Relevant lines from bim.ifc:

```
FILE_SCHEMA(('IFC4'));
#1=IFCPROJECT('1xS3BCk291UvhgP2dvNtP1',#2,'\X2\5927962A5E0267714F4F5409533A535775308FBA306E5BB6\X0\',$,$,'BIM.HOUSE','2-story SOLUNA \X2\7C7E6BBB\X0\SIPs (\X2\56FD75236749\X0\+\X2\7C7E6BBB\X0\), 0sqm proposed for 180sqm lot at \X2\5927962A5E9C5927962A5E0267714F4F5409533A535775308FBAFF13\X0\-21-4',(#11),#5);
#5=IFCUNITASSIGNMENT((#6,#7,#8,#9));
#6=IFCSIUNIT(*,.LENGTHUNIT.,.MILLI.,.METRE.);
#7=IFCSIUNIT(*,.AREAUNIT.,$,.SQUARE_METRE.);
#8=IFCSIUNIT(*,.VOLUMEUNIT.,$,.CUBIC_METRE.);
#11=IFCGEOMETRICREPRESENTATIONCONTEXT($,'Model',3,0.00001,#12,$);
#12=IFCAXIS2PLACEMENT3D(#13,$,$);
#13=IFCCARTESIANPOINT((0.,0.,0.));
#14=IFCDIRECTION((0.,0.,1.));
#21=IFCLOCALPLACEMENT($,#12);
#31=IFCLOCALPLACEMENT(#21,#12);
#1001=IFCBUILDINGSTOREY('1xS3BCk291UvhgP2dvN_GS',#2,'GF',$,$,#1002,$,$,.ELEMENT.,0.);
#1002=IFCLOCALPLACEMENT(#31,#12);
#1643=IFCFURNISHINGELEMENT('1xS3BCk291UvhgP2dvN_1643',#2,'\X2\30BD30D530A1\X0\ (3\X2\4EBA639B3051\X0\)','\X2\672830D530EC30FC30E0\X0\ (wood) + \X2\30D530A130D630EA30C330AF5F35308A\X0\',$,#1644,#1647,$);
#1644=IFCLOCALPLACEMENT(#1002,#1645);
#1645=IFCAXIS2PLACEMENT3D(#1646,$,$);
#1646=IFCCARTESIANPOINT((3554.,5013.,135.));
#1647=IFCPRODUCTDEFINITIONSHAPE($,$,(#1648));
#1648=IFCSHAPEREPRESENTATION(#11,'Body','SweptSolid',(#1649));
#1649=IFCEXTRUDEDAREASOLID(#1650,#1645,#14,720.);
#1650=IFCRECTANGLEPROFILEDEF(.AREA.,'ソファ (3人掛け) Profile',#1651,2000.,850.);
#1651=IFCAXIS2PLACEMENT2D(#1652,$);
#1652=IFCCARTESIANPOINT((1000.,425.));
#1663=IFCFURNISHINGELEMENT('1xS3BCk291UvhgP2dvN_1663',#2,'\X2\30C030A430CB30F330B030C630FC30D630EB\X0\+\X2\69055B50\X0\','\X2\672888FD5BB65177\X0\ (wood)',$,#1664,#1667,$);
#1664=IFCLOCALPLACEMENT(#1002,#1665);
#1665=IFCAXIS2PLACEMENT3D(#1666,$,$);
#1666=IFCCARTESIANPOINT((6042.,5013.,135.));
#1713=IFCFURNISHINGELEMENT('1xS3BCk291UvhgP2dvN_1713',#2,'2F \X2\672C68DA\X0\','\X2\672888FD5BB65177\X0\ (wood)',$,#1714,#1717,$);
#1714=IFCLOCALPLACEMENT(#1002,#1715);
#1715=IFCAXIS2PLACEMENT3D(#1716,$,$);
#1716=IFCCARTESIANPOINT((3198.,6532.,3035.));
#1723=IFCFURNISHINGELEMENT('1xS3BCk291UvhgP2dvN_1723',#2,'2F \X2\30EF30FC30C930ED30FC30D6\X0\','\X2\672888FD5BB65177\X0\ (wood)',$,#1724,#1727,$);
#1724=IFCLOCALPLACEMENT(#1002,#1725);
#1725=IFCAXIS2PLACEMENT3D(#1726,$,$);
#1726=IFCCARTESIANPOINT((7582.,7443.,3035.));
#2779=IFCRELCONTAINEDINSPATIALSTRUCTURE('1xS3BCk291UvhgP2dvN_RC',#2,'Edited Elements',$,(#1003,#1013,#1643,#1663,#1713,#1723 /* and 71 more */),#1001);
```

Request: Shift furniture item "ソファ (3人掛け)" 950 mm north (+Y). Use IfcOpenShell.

```python
import ifcopenshell
import ifcopenshell.api.geometry
import ifcopenshell.util.placement
import ifcopenshell.util.unit

model = ifcopenshell.open("bim.ifc")
unit_scale = ifcopenshell.util.unit.calculate_unit_scale(model)

item = model.by_guid("1xS3BCk291UvhgP2dvN_1643")
matrix = ifcopenshell.util.placement.get_local_placement(item.ObjectPlacement)
matrix[1, 3] += 0.95 / unit_scale
ifcopenshell.api.geometry.edit_object_placement(model, product=item, matrix=matrix, is_si=False)

print(ifcopenshell.util.placement.get_local_placement(item.ObjectPlacement).round(3) + 0.0)

model.write("bim_updated.ifc")
```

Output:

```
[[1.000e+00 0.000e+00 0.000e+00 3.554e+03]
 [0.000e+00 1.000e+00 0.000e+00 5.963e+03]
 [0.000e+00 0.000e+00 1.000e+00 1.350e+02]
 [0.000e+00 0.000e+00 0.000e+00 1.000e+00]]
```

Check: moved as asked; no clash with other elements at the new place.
